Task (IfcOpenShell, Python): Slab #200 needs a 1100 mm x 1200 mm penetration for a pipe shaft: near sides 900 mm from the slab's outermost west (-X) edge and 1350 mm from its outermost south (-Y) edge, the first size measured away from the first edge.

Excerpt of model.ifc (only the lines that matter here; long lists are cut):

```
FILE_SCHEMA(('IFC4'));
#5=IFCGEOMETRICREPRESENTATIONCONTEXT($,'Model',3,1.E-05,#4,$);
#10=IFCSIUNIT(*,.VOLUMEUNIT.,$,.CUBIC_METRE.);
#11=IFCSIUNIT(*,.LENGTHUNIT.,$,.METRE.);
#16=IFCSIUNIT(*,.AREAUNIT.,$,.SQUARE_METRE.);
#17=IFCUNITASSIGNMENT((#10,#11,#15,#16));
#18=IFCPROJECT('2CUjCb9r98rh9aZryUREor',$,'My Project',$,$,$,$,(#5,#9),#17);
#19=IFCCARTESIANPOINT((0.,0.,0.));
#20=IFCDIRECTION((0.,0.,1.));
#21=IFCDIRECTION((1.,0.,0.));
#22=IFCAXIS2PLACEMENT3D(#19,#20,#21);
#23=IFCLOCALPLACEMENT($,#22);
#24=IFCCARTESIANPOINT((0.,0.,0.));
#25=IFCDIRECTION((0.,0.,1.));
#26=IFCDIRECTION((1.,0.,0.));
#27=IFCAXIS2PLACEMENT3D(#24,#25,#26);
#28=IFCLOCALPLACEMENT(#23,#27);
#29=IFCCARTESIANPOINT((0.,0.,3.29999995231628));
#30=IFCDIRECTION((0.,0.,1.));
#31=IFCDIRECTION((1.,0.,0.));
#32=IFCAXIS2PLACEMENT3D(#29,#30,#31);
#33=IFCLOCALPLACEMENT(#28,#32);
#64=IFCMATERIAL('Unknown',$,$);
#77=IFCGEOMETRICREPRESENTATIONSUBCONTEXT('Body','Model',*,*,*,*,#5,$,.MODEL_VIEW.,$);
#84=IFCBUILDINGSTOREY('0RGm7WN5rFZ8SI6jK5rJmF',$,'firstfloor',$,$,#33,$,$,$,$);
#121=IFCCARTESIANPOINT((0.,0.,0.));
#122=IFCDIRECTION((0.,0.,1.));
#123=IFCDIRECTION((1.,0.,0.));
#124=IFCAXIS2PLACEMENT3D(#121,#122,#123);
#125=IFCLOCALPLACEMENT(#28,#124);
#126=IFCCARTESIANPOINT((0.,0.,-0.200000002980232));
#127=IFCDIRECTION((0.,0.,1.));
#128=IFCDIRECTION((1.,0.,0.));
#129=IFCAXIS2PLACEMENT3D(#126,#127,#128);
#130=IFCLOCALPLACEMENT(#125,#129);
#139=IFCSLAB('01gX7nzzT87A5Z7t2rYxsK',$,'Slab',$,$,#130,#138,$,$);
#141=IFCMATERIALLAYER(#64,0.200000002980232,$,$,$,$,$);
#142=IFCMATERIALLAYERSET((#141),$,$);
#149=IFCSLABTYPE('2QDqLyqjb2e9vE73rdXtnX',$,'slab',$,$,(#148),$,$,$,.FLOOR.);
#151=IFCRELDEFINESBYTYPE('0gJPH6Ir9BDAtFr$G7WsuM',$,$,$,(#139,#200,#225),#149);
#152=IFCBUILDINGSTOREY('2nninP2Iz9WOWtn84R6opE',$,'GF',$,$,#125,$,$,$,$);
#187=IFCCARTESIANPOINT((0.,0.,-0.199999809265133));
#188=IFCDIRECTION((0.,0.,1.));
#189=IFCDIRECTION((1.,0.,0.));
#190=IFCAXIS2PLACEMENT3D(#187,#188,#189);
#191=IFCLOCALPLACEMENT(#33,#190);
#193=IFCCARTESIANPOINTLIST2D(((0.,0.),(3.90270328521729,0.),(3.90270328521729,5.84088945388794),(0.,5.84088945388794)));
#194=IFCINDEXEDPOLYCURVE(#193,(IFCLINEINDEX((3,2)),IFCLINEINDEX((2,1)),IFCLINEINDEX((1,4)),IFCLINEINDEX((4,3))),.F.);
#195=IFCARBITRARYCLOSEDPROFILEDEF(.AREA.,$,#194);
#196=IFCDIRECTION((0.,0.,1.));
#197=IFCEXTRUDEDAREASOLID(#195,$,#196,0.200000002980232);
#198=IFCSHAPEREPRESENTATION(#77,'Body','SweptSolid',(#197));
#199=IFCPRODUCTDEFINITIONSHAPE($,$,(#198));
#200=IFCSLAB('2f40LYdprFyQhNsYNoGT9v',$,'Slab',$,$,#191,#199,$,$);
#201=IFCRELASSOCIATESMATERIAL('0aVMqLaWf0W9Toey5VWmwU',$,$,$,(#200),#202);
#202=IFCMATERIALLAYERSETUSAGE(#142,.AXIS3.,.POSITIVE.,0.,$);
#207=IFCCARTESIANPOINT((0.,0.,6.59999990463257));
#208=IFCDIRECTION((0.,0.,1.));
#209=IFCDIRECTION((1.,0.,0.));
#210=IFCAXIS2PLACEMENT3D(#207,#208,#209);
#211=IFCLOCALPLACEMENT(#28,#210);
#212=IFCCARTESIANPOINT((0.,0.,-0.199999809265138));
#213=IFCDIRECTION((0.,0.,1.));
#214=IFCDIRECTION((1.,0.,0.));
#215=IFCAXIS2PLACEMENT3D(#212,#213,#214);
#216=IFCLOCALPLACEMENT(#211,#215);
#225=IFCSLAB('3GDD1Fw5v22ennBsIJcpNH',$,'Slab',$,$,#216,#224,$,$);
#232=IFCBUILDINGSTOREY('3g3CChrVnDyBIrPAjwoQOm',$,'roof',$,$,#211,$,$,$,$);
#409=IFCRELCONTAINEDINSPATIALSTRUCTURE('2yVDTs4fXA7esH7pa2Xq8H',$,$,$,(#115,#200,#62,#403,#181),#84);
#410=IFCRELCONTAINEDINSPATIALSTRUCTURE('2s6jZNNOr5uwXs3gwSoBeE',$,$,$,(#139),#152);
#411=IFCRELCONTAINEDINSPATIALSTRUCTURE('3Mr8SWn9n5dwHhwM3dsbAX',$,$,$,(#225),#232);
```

```python
import numpy as np
import ifcopenshell
import ifcopenshell.api.feature
import ifcopenshell.api.geometry
import ifcopenshell.api.root
import ifcopenshell.geom
import ifcopenshell.util.placement
import ifcopenshell.util.representation
import ifcopenshell.util.shape
import ifcopenshell.util.unit

model = ifcopenshell.open("model.ifc")
unit_scale = ifcopenshell.util.unit.calculate_unit_scale(model)
settings = ifcopenshell.geom.settings()


def volume(element):
    """Net volume in cubic metres, openings subtracted."""
    shape = ifcopenshell.geom.create_shape(settings, element)
    return ifcopenshell.util.shape.get_volume(shape.geometry)


slab = model.by_guid("2f40LYdprFyQhNsYNoGT9v")
before = volume(slab)

# Extent in the slab's own axes, in metres. The edges named are its -X and -Y sides.
slab_shape = ifcopenshell.geom.create_shape(settings, slab)
vertices = ifcopenshell.util.shape.get_vertices(slab_shape.geometry)
x_min, y_min, bottom = vertices.min(axis=0)
top = vertices[:, 2].max()

opening = ifcopenshell.api.root.create_entity(model, ifc_class="IfcOpeningElement", name="Pipe shaft opening", predefined_type="OPENING")
context = ifcopenshell.util.representation.get_context(model, "Model", "Body", "MODEL_VIEW")
width, depth = 1.1, 1.2
outline = [(0.0, 0.0), (width, 0.0), (width, depth), (0.0, depth), (0.0, 0.0)]
# Overshoot both faces by 50 mm so the cut is clean.
shape = ifcopenshell.api.geometry.add_slab_representation(
    model, context=context, depth=top - bottom + 0.1, polyline=outline
)
ifcopenshell.api.geometry.assign_representation(model, product=opening, representation=shape)

matrix = ifcopenshell.util.placement.get_local_placement(slab.ObjectPlacement)
matrix[:, 3] = matrix @ np.append(np.array([x_min + 0.9, y_min + 1.35, bottom - 0.05]) / unit_scale, 1.0)
ifcopenshell.api.geometry.edit_object_placement(model, product=opening, matrix=matrix, is_si=False)
ifcopenshell.api.feature.add_feature(model, feature=opening, element=slab)

after = volume(slab)

print(f"slab volume {before:.3f} -> {after:.3f} m3")

model.write("model-out.ifc")
```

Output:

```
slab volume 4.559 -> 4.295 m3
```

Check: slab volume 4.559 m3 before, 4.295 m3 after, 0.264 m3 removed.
